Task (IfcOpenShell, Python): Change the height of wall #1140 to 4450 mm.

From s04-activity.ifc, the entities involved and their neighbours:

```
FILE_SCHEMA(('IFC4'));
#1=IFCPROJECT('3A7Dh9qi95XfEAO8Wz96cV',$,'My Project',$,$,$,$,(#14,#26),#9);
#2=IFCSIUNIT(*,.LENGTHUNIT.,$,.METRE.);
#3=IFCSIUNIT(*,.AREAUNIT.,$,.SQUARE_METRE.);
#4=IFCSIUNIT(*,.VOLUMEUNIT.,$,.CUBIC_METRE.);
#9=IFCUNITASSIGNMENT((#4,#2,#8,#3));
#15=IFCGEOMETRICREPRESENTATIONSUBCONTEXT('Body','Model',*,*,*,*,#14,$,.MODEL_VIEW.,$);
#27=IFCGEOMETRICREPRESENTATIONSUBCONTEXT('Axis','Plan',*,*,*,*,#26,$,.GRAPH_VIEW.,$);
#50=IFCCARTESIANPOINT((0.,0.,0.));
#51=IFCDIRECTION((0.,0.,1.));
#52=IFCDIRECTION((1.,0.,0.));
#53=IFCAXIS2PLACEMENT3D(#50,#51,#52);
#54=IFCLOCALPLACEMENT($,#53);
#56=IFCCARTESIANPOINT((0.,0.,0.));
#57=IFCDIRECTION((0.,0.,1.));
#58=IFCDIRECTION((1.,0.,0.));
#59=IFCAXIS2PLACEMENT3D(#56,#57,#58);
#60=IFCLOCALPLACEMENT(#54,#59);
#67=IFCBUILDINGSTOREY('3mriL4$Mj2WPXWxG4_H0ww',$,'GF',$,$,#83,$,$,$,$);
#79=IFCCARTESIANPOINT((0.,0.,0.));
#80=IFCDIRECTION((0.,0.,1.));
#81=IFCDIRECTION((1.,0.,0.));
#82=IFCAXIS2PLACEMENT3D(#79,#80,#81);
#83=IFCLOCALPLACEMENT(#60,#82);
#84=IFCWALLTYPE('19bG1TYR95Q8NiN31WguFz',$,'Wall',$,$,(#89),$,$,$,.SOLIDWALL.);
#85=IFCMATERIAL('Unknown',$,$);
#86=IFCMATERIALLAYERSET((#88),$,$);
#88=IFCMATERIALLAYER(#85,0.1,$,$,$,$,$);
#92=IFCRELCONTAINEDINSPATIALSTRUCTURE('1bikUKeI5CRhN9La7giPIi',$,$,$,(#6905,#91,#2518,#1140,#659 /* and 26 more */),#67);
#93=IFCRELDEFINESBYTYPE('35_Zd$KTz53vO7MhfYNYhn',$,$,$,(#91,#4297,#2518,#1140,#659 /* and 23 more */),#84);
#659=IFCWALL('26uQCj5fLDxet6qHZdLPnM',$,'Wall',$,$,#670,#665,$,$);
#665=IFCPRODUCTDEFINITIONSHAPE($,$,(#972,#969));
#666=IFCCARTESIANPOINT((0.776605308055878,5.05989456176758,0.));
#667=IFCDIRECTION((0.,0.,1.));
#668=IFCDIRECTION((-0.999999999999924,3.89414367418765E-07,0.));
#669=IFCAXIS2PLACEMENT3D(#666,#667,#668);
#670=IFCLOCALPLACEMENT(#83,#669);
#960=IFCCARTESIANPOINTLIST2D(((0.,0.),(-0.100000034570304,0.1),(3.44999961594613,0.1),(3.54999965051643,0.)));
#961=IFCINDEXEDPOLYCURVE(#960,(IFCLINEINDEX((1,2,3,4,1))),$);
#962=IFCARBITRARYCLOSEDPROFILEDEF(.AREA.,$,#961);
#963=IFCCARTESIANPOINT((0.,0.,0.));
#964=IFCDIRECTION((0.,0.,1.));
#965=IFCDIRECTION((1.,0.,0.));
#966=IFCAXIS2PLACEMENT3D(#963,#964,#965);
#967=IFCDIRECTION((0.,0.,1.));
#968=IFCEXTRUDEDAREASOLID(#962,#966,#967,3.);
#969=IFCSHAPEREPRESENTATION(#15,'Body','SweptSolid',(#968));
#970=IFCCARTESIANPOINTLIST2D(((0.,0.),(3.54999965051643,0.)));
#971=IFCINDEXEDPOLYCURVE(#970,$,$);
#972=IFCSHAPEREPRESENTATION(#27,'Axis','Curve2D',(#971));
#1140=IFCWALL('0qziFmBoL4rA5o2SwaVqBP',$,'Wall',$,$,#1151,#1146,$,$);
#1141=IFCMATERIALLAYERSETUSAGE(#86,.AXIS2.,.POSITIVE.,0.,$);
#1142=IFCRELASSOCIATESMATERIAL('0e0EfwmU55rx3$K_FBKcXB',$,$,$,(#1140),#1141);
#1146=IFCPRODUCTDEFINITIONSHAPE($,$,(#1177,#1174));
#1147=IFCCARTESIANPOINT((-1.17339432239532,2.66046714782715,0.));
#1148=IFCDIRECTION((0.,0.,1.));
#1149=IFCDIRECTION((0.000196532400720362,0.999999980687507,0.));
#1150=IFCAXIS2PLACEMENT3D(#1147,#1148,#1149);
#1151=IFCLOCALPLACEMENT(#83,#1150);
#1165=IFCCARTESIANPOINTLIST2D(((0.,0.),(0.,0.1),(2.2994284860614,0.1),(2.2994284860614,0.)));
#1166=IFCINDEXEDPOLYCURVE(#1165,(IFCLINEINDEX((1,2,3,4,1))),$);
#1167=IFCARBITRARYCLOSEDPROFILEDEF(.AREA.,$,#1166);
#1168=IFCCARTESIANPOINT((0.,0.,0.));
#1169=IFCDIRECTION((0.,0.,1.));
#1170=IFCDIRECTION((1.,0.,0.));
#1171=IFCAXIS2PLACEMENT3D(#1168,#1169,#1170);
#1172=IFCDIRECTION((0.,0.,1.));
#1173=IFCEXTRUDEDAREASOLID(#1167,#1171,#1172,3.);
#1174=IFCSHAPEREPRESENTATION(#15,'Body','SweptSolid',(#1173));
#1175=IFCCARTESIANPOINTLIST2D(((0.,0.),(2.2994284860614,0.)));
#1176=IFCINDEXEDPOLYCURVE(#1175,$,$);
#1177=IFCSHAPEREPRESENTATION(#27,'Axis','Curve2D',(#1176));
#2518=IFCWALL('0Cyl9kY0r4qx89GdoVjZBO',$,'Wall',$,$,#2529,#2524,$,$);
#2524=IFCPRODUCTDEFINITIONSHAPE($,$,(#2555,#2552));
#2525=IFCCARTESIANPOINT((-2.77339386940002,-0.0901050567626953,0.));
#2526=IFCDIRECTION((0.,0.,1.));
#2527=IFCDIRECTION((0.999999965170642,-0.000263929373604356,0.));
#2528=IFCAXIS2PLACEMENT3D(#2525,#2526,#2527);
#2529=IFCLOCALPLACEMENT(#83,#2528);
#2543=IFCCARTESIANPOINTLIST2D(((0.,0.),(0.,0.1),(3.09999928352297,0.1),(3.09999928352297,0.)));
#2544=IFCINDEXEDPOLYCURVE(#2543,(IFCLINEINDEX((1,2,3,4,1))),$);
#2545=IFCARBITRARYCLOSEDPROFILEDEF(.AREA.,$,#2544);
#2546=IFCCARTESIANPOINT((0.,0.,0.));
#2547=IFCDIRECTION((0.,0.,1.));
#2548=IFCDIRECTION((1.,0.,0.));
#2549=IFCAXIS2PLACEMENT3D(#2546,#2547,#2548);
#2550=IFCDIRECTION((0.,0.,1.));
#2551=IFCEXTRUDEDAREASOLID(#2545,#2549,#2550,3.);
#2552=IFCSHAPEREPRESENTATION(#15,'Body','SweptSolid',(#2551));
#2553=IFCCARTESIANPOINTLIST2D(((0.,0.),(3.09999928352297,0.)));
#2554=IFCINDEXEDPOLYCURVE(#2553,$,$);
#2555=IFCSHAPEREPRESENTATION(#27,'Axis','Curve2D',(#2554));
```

```python
import ifcopenshell
import ifcopenshell.geom
import ifcopenshell.util.representation
import ifcopenshell.util.shape
import ifcopenshell.util.unit

model = ifcopenshell.open("s04-activity.ifc")
unit_scale = ifcopenshell.util.unit.calculate_unit_scale(model)
settings = ifcopenshell.geom.settings()


def volume(element):
    """Net volume in cubic metres, openings subtracted."""
    shape = ifcopenshell.geom.create_shape(settings, element)
    return ifcopenshell.util.shape.get_volume(shape.geometry)


wall = model.by_guid("0qziFmBoL4rA5o2SwaVqBP")
before = volume(wall)

body = ifcopenshell.util.representation.get_representation(wall, "Model", "Body")
solid = body.Items[0]
old_height = solid.Depth
solid.Depth = 4.45 / unit_scale
after = volume(wall)

print(f"height {old_height:g} -> {solid.Depth:g}, volume {before:.3f} -> {after:.3f} m3")

model.write("s04-activity-out.ifc")
```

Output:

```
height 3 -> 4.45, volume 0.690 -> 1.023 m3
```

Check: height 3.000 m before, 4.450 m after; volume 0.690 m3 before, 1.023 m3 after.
